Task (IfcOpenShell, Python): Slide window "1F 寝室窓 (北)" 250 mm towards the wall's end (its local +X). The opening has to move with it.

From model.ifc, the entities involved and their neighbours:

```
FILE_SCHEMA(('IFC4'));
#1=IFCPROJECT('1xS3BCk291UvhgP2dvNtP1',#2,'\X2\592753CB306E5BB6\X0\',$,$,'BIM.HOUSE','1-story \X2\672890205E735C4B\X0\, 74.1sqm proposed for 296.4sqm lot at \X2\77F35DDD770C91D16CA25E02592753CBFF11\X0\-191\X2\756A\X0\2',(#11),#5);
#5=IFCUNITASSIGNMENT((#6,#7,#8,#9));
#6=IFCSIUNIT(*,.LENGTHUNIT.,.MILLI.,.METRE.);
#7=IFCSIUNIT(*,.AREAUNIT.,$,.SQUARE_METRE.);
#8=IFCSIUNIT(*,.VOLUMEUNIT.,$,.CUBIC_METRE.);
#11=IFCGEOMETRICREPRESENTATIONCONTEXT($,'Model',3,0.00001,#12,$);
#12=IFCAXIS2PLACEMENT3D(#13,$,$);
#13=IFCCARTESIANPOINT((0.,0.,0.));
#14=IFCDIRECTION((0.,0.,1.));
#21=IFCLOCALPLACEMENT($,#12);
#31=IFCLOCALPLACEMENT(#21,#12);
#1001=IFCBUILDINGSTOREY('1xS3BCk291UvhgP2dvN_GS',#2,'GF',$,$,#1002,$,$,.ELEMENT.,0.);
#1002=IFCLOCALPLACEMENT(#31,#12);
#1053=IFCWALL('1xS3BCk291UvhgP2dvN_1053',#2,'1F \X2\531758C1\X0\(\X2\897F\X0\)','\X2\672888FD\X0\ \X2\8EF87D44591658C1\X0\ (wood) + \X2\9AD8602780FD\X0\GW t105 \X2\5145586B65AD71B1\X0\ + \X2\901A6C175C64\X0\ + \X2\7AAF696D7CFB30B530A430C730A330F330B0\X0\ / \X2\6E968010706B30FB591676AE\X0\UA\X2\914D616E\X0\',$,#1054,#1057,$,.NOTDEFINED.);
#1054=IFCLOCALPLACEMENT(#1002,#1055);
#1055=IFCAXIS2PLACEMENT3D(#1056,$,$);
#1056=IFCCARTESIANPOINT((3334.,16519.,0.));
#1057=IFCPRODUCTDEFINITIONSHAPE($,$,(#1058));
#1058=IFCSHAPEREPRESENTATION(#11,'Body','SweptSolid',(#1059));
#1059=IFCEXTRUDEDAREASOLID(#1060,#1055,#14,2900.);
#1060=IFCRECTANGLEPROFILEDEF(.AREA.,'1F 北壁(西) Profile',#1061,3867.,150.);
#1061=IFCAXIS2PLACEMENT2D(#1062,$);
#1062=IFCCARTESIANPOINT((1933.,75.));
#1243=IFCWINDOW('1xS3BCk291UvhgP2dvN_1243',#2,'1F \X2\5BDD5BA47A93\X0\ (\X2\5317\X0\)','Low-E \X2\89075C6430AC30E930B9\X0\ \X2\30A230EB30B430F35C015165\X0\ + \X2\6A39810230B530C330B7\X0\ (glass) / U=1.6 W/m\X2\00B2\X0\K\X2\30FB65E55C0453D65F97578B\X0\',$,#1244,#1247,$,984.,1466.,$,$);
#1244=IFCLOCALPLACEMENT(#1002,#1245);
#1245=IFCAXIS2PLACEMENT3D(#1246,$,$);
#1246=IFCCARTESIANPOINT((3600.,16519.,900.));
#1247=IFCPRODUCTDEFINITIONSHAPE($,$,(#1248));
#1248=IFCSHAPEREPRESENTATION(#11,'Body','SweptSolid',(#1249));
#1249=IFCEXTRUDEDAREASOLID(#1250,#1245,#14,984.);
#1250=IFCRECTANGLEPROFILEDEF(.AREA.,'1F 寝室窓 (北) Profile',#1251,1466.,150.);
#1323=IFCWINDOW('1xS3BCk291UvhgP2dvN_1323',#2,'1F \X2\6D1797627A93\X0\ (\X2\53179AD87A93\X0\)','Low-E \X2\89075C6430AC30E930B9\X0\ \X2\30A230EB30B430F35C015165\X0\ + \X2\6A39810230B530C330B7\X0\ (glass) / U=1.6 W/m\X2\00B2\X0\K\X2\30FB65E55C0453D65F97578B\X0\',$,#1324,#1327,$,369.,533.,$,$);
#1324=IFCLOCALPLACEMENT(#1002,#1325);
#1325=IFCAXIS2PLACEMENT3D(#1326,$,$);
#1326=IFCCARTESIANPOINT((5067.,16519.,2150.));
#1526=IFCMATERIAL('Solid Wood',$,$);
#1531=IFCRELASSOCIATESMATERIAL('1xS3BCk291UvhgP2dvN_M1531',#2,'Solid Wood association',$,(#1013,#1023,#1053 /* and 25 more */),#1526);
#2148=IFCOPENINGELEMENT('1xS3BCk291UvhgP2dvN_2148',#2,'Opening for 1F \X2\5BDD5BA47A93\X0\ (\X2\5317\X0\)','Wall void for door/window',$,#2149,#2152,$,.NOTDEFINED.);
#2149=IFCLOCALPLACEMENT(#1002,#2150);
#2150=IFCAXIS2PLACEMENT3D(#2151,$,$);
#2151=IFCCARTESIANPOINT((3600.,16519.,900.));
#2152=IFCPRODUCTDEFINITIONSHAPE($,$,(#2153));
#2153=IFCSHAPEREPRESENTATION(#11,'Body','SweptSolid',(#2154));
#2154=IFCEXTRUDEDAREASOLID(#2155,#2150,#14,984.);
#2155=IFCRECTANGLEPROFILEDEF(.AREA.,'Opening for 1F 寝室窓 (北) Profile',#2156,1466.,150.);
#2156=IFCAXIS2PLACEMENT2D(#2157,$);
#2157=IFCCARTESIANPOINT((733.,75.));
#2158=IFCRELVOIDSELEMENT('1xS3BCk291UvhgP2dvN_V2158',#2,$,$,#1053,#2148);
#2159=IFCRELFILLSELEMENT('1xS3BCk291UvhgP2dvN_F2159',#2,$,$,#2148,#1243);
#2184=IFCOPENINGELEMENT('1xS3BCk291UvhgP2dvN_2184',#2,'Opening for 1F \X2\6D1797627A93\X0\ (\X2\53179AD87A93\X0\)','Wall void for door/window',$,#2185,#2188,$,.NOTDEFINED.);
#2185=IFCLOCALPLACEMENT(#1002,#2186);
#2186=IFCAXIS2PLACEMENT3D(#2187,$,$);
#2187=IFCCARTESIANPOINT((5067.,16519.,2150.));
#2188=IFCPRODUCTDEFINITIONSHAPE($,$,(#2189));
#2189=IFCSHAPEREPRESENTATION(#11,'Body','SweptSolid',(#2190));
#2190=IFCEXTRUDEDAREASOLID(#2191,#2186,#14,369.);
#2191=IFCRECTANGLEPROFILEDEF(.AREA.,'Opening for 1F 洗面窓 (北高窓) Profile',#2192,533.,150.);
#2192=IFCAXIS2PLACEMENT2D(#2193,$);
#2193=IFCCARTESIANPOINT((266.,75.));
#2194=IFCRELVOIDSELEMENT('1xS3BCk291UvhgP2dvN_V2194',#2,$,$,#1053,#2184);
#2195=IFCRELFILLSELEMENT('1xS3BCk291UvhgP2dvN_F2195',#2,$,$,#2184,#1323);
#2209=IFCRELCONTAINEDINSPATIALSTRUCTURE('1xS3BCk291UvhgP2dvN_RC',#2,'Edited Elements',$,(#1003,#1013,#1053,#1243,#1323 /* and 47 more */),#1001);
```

```python
import ifcopenshell
import ifcopenshell.api.geometry
import ifcopenshell.util.placement
import ifcopenshell.util.unit

model = ifcopenshell.open("model.ifc")
unit_scale = ifcopenshell.util.unit.calculate_unit_scale(model)

window = model.by_id(1243)
opening = window.FillsVoids[0].RelatingOpeningElement
wall = opening.VoidsElements[0].RelatingBuildingElement

wall_matrix = ifcopenshell.util.placement.get_local_placement(wall.ObjectPlacement)
shift = wall_matrix[:3, 0] * 0.25 / unit_scale
before = ifcopenshell.util.placement.get_local_placement(window.ObjectPlacement)[:3, 3].copy()

# The window is not placed relative to its opening, so move both.
for product in (opening, window):
    matrix = ifcopenshell.util.placement.get_local_placement(product.ObjectPlacement)
    matrix[:3, 3] += shift
    ifcopenshell.api.geometry.edit_object_placement(model, product=product, matrix=matrix, is_si=False)

after = ifcopenshell.util.placement.get_local_placement(window.ObjectPlacement)[:3, 3]
print("window moved by", (after - before).round(3) + 0.0)

model.write("model_updated.ifc")
```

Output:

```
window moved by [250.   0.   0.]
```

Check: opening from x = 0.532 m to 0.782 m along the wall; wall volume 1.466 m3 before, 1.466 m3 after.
